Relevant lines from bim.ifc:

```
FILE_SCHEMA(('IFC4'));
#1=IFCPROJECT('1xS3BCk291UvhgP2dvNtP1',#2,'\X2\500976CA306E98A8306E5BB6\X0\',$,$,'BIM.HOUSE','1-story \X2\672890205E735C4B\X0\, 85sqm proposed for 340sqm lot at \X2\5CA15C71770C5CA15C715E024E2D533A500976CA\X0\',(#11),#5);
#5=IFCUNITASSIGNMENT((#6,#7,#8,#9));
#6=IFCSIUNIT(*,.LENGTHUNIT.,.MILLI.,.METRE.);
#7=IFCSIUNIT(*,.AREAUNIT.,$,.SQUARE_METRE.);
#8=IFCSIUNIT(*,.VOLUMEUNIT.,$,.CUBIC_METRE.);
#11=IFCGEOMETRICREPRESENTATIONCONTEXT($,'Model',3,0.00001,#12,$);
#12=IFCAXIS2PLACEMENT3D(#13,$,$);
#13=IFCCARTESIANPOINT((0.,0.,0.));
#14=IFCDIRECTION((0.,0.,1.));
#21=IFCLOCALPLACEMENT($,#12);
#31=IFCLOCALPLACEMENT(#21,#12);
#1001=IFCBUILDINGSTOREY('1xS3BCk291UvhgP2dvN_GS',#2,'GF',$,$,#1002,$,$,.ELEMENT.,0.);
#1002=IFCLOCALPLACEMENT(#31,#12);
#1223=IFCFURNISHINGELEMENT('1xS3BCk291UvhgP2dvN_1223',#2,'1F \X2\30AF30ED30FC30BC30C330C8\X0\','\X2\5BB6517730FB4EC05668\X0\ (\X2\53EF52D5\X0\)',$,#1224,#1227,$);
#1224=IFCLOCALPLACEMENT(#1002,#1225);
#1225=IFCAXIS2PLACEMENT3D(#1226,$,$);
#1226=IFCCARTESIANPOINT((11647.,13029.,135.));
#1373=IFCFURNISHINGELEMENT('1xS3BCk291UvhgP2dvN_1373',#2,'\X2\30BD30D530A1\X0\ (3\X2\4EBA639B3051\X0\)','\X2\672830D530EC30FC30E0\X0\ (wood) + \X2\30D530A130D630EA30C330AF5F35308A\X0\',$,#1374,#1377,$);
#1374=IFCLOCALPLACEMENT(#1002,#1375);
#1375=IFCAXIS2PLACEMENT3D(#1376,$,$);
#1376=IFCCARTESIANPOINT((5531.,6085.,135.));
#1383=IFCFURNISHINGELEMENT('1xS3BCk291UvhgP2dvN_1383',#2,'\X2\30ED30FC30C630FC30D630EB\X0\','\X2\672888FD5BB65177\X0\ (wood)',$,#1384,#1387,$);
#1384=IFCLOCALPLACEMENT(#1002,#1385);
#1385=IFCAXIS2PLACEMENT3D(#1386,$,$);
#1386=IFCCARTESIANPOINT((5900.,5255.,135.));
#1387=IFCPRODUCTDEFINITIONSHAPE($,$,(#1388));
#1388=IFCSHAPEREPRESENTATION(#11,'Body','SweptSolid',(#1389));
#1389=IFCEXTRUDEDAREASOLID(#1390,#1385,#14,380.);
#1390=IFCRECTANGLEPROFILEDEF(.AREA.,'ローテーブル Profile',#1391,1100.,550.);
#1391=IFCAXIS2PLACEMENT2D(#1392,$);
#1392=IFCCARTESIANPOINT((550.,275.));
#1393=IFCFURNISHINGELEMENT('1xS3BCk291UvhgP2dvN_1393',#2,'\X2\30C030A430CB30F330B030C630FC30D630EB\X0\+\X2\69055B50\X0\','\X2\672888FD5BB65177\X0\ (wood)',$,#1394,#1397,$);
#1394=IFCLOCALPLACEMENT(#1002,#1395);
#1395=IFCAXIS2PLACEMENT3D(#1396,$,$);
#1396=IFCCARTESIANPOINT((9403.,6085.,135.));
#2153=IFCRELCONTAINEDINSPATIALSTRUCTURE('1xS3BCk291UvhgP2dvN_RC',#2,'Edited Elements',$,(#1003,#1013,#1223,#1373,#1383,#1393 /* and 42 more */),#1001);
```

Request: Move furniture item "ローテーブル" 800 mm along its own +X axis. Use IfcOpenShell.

```python
import ifcopenshell
import ifcopenshell.api.geometry
import ifcopenshell.util.placement

model = ifcopenshell.open("bim.ifc")

item = model.by_id(1383)
matrix = ifcopenshell.util.placement.get_local_placement(item.ObjectPlacement)
matrix[:3, 3] += matrix[:3, 0] * 800.0
ifcopenshell.api.geometry.edit_object_placement(model, product=item, matrix=matrix, is_si=False)

print(ifcopenshell.util.placement.get_local_placement(item.ObjectPlacement).round(3) + 0.0)

model.write("bim_rev.ifc")
```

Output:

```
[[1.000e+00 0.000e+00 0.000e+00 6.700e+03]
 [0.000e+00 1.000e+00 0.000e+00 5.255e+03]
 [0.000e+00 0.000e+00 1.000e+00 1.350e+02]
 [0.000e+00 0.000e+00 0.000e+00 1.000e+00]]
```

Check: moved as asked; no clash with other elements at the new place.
